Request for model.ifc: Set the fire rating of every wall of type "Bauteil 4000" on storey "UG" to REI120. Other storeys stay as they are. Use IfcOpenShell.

First a look at what the model holds.

```python
import ifcopenshell
import ifcopenshell.util.element

model = ifcopenshell.open("model.ifc")
print(model.schema)
storey = next(s for s in model.by_type("IfcBuildingStorey") if s.Name == "UG")
walls = [e for e in ifcopenshell.util.element.get_decomposition(storey) if e.is_a("IfcWall")]
seen = {}
for e in walls:
    element_type = ifcopenshell.util.element.get_type(e)
    key = (element_type.Name if element_type != e and element_type else None, ifcopenshell.util.element.get_pset(e, "Pset_WallCommon", "FireRating"))
    seen[key] = seen.get(key, 0) + 1
for (name, value), count in sorted(seen.items(), key=str):
    print(count, "x", name, "|", value)
```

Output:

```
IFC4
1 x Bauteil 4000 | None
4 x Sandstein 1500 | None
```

```python
import ifcopenshell
import ifcopenshell.api.pset
import ifcopenshell.util.element

model = ifcopenshell.open("model.ifc")

storey = next(s for s in model.by_type("IfcBuildingStorey") if s.Name == "UG")
walls = [e for e in ifcopenshell.util.element.get_decomposition(storey) if e.is_a("IfcWall")]

count = 0
for e in walls:
    element_type = ifcopenshell.util.element.get_type(e)
    if element_type in (None, e) or element_type.Name != "Bauteil 4000":
        continue
    # add_pset returns the element's existing set when there is one.
    pset = ifcopenshell.api.pset.add_pset(model, product=e, name="Pset_WallCommon")
    ifcopenshell.api.pset.edit_pset(model, pset=pset, properties={"FireRating": "REI120"})
    count += 1

print(count, "walls updated")

model.write("model_rev.ifc")
```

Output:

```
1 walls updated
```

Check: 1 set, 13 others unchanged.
